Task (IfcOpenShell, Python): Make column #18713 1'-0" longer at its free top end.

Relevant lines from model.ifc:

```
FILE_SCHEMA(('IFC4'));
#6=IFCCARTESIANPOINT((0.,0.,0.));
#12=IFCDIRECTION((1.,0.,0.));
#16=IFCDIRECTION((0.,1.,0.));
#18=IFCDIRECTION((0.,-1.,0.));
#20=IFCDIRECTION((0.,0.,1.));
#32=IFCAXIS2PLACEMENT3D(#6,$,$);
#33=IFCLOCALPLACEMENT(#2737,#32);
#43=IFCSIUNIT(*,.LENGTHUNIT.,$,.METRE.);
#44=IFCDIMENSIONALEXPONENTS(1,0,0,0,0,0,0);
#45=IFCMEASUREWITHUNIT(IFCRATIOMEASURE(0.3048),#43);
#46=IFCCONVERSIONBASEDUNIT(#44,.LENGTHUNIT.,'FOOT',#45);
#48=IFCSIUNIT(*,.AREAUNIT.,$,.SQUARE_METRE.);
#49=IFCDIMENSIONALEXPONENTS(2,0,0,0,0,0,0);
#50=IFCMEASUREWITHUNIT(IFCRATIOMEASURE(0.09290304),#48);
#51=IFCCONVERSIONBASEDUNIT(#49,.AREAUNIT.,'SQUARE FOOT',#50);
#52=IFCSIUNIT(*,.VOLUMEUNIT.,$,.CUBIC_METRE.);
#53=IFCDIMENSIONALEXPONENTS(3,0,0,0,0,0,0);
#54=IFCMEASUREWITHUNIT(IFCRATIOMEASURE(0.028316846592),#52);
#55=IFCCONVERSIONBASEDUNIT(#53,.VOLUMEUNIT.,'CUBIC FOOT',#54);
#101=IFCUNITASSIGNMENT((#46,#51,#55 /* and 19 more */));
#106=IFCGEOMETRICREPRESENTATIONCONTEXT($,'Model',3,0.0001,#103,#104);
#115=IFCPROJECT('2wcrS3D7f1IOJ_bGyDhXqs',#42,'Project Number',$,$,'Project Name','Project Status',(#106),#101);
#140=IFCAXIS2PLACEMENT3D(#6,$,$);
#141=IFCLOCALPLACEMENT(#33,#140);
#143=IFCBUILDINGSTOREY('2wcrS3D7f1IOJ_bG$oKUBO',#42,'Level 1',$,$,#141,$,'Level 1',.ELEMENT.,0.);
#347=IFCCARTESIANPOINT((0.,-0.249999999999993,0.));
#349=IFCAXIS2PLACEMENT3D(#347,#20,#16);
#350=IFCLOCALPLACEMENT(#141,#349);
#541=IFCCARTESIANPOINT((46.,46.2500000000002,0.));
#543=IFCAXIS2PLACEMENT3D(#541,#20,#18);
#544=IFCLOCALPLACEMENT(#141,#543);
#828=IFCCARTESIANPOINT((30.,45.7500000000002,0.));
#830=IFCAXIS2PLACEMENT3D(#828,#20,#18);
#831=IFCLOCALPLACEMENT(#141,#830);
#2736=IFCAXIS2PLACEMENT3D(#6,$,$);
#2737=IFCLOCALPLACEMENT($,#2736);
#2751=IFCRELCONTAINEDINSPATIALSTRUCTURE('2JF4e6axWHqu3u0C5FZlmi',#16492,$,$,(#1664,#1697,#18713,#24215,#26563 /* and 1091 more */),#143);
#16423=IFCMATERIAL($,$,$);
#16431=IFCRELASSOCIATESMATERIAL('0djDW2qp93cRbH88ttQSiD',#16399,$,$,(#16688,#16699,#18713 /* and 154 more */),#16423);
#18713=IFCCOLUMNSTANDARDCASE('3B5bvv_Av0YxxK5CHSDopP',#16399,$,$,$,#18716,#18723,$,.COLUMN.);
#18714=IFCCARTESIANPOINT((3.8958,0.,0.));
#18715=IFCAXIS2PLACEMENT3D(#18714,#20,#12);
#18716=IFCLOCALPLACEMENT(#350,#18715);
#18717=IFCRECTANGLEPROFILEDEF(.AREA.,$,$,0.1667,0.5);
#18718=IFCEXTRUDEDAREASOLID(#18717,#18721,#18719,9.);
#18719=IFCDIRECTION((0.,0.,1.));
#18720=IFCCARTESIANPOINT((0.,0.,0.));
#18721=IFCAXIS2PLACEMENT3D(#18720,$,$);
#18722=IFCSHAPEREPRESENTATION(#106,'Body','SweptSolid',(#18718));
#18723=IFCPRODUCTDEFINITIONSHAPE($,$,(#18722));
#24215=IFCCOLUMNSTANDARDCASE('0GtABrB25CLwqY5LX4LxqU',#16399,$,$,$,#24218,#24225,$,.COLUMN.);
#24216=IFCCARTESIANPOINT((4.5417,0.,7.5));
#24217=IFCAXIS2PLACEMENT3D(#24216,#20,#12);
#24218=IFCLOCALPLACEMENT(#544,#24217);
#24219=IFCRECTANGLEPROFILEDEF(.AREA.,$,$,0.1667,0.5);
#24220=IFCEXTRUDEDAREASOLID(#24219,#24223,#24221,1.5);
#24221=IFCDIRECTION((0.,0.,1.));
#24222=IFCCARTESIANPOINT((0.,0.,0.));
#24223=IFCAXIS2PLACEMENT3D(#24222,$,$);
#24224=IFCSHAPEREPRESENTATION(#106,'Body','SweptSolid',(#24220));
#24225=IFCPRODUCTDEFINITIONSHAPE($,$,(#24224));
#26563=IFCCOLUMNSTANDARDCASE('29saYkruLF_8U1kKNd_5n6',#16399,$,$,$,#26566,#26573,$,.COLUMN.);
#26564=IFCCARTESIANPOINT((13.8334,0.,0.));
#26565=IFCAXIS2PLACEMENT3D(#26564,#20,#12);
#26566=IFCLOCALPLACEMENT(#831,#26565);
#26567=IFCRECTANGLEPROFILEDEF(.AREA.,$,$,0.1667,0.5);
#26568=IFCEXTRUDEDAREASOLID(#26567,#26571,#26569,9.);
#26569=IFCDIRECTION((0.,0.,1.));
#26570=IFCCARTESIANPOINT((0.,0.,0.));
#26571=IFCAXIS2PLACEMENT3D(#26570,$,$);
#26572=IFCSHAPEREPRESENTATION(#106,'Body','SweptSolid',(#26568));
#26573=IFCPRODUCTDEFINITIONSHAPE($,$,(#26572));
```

```python
import ifcopenshell
import ifcopenshell.util.unit

model = ifcopenshell.open("model.ifc")
unit_scale = ifcopenshell.util.unit.calculate_unit_scale(model)

member = model.by_guid("3B5bvv_Av0YxxK5CHSDopP")
change = 12 * 0.0254 / unit_scale

# The extrusion runs towards the end named, so only its depth changes.
body = next(r for r in member.Representation.Representations if r.RepresentationIdentifier == "Body")
solid = body.Items[0]
old_length = solid.Depth
solid.Depth += change

print(f"length {old_length:g} -> {solid.Depth:g}")

model.write("model_v2.ifc")
```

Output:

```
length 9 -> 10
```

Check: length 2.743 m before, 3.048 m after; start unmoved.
